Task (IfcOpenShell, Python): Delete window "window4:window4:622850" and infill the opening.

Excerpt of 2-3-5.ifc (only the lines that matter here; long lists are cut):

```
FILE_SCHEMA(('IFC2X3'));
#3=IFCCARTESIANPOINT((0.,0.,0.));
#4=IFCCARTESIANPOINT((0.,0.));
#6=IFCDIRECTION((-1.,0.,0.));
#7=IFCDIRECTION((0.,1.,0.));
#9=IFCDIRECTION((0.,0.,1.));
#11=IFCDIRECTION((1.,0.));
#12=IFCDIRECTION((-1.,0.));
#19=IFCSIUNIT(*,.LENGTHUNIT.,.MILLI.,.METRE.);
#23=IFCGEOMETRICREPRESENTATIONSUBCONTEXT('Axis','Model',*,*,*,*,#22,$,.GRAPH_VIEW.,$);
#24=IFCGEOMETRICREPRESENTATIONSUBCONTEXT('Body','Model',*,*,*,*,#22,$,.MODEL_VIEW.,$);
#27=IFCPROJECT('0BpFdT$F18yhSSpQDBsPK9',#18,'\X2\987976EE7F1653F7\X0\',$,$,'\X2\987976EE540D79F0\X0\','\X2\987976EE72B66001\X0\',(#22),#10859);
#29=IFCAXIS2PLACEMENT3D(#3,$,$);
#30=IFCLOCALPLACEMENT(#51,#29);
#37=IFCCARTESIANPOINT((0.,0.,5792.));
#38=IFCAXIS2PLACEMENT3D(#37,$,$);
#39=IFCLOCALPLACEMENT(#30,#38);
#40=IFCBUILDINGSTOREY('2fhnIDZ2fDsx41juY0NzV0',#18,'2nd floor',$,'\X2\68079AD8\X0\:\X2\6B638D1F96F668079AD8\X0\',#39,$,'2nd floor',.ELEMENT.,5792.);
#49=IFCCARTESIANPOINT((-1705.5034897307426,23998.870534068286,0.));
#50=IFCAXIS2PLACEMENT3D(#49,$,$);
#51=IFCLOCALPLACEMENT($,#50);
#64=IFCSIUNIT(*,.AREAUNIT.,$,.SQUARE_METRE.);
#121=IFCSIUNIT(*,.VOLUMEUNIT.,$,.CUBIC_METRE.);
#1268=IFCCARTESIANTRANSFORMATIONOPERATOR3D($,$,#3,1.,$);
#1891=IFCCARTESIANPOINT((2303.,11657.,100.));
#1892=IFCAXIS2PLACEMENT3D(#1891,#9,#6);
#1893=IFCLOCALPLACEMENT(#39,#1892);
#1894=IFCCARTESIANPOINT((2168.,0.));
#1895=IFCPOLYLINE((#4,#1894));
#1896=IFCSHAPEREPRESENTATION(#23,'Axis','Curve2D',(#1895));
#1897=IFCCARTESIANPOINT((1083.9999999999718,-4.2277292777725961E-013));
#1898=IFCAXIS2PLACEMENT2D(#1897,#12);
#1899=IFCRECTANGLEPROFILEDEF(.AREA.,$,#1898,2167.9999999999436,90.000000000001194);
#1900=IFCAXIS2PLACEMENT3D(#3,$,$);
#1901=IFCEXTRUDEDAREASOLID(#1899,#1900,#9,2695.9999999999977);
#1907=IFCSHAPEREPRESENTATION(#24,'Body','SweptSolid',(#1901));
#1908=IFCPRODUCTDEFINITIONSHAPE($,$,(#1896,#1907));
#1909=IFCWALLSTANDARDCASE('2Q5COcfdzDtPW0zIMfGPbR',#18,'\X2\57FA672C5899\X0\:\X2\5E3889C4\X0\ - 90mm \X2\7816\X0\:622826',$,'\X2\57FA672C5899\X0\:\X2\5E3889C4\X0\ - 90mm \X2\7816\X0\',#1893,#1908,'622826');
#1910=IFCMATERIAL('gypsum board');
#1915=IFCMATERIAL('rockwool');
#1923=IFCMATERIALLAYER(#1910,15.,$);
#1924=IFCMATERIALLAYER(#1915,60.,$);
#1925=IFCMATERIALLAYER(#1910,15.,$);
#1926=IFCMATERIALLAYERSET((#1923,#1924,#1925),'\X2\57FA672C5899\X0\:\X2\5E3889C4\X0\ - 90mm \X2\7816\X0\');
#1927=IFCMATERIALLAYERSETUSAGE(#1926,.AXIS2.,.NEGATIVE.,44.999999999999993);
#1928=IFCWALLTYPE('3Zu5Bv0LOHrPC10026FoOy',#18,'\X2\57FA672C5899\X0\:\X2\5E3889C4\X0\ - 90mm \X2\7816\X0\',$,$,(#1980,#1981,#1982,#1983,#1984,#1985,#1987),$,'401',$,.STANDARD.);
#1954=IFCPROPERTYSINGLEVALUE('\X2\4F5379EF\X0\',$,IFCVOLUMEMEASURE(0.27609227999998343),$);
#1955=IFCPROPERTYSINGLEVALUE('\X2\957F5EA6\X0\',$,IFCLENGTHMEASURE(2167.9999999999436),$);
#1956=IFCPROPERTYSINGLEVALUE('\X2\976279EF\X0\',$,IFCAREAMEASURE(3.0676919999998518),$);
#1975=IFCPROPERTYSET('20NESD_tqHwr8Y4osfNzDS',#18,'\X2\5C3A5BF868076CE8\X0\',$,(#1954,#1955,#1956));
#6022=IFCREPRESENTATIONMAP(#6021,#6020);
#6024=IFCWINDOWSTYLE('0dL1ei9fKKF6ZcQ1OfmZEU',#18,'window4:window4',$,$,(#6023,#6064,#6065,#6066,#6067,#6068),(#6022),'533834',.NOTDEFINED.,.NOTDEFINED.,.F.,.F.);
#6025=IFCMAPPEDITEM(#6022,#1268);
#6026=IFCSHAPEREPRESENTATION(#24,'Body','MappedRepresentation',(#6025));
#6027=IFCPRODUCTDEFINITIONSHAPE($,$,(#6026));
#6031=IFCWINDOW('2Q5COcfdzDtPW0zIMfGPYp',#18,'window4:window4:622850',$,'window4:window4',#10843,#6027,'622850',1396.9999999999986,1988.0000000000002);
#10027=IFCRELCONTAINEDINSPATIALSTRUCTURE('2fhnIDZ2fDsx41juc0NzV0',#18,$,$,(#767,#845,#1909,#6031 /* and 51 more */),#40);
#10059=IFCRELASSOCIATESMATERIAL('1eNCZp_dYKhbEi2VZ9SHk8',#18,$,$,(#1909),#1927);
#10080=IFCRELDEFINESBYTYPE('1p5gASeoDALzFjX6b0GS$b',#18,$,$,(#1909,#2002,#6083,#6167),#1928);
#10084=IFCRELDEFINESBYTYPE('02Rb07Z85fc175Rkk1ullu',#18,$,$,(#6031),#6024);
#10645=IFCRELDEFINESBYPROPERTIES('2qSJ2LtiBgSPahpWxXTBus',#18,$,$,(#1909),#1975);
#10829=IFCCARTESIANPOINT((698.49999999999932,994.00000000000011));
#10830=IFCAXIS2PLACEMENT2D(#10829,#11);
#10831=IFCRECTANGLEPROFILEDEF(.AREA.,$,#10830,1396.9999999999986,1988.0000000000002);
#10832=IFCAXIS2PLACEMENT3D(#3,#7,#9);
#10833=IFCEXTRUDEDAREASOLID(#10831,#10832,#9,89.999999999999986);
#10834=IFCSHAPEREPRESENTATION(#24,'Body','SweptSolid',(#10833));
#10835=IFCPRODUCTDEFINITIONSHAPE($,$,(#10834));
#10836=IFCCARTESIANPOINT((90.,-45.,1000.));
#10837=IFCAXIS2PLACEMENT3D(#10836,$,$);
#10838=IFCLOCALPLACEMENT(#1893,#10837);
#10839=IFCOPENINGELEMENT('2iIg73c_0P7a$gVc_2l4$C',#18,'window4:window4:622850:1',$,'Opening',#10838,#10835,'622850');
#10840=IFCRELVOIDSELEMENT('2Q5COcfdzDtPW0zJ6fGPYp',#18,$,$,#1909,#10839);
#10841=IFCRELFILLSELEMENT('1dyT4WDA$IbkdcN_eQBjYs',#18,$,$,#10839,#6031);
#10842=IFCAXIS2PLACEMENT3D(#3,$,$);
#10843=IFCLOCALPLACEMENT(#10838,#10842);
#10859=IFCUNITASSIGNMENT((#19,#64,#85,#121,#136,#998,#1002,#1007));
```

```python
import ifcopenshell
import ifcopenshell.api.feature
import ifcopenshell.api.pset
import ifcopenshell.api.root
import ifcopenshell.geom
import ifcopenshell.util.element
import ifcopenshell.util.shape
import ifcopenshell.util.unit

model = ifcopenshell.open("2-3-5.ifc")
area_scale = ifcopenshell.util.unit.calculate_unit_scale(model, "AREAUNIT")
volume_scale = ifcopenshell.util.unit.calculate_unit_scale(model, "VOLUMEUNIT")
settings = ifcopenshell.geom.settings()


def volume(element):
    """Net volume in cubic metres, openings subtracted."""
    shape = ifcopenshell.geom.create_shape(settings, element)
    return ifcopenshell.util.shape.get_volume(shape.geometry)


window = model.by_id(6031)
opening = window.FillsVoids[0].RelatingOpeningElement
wall = opening.VoidsElements[0].RelatingBuildingElement
before = volume(wall)

ifcopenshell.api.root.remove_product(model, product=window)
ifcopenshell.api.feature.remove_feature(model, feature=opening)

after = volume(wall)
thickness = 0.09  # wall thickness in metres

# Update the wall's stored quantities.
pset = model.by_id(ifcopenshell.util.element.get_pset(wall, "尺寸标注", should_inherit=False)["id"])
ifcopenshell.api.pset.edit_pset(model, pset=pset, properties={
    "体积": model.create_entity("IfcVolumeMeasure", after / volume_scale),
    "面积": model.create_entity("IfcAreaMeasure", after / thickness / area_scale),
})

print(f"wall volume {before:.3f} -> {after:.3f} m3")

model.write("2-3-5-out.ifc")
```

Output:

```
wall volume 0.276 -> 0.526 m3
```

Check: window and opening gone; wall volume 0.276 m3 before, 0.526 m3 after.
